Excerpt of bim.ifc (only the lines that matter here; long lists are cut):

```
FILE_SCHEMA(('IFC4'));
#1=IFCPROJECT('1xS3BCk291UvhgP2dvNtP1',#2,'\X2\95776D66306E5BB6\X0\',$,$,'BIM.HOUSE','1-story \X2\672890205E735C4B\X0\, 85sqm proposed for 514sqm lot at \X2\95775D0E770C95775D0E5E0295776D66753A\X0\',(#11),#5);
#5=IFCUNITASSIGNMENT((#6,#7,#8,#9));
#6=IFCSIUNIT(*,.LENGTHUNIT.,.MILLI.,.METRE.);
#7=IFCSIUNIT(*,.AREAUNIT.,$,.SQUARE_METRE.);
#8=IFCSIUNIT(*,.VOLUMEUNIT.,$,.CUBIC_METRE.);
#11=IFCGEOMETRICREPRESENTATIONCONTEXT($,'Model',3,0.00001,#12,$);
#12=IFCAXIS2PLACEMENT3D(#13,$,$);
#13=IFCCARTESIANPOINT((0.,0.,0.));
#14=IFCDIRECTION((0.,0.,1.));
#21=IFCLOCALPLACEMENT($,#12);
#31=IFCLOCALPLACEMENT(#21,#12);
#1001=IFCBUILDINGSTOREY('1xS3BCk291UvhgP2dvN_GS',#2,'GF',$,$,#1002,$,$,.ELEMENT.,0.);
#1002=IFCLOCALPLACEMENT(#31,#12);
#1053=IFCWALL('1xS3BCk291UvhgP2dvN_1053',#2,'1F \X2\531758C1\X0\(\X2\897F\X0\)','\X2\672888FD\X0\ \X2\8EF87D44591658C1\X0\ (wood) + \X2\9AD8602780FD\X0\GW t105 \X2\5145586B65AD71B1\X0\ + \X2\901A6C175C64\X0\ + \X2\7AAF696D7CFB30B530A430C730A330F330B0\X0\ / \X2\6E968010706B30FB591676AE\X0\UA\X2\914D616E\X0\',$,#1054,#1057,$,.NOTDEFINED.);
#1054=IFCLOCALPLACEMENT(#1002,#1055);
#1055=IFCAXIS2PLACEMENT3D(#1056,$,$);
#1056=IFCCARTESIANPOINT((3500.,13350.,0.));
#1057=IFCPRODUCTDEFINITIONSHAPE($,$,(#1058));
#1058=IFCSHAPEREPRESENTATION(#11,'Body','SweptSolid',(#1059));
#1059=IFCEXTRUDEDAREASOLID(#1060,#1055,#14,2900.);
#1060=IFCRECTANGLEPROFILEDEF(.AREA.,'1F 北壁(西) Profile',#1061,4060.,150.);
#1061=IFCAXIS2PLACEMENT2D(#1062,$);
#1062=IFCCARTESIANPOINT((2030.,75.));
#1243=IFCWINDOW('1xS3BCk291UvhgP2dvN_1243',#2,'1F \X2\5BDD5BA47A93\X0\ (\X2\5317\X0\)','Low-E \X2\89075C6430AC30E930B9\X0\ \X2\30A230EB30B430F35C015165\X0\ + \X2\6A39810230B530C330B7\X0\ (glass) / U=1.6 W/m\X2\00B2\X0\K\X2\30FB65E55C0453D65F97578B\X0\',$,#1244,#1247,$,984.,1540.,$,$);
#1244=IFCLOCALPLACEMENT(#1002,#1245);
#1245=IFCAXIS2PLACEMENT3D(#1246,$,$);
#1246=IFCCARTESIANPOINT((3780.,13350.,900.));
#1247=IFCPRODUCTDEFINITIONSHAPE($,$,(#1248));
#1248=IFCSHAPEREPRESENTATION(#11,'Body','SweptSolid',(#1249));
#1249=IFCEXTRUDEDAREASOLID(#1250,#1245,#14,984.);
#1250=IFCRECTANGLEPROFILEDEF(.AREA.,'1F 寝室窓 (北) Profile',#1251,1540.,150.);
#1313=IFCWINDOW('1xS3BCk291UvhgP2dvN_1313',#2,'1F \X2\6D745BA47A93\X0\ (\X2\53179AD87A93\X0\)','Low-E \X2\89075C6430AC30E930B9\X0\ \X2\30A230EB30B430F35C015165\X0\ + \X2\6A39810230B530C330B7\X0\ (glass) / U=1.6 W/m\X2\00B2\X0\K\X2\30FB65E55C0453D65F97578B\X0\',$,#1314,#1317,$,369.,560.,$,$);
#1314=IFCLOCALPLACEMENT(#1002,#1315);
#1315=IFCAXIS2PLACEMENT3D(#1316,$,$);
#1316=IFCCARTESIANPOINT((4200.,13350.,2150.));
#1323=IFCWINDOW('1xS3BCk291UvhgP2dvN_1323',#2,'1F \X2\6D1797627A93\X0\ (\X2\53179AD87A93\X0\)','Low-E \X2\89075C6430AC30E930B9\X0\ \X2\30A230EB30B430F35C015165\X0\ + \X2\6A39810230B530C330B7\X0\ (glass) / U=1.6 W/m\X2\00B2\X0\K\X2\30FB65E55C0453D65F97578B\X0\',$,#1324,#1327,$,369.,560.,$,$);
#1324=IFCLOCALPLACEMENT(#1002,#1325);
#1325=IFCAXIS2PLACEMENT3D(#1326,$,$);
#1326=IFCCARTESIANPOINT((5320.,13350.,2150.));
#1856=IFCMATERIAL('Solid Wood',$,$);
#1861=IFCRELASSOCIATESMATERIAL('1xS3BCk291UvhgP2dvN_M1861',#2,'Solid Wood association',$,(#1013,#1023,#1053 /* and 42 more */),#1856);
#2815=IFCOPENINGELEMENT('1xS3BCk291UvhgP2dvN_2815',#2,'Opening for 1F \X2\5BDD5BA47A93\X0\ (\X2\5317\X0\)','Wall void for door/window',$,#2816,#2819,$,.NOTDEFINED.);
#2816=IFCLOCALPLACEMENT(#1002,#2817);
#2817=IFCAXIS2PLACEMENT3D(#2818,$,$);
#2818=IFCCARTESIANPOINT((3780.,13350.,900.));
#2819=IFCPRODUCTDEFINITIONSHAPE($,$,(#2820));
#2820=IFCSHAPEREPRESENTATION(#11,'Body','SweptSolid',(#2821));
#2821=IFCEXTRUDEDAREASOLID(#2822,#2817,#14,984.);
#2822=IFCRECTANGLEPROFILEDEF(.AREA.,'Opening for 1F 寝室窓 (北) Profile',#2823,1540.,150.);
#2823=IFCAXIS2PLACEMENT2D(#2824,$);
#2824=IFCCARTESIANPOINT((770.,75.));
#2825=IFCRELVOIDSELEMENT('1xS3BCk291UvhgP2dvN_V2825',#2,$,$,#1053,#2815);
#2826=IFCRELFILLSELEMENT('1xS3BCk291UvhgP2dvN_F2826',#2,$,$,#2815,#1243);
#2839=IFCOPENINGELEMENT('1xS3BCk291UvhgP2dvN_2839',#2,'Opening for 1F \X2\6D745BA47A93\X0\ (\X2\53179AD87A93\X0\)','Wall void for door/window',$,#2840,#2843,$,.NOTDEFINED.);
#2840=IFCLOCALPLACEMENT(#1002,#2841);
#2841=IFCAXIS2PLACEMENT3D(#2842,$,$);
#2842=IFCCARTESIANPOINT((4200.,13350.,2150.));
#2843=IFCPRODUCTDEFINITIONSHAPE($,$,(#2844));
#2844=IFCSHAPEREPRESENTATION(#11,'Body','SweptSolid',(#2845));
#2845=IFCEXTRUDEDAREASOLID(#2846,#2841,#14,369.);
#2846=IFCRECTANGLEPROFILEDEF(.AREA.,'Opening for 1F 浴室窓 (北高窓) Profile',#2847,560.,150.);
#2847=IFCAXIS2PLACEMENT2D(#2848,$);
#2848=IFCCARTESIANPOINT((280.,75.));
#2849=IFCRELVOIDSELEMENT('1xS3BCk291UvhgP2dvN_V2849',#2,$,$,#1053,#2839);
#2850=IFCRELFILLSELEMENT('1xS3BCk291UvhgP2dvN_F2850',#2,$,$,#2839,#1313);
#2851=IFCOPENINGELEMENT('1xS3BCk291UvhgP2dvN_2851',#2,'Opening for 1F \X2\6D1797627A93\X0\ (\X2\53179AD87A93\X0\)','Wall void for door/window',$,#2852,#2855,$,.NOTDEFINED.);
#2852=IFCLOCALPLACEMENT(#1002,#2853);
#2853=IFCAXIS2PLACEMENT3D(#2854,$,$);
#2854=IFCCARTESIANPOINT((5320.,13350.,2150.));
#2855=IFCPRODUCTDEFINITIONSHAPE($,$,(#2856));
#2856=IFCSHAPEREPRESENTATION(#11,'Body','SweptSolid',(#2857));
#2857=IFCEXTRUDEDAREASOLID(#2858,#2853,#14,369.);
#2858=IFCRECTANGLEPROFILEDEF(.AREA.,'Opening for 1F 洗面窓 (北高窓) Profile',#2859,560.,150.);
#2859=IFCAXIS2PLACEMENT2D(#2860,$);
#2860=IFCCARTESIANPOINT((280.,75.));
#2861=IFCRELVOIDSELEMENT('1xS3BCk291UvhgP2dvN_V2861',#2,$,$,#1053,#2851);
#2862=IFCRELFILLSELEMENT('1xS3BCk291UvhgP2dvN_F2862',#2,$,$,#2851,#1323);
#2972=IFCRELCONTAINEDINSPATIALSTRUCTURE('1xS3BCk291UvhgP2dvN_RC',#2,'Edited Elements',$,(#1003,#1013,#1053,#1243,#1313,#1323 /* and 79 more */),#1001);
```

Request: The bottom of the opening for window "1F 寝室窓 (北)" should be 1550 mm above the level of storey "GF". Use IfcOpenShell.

```python
import numpy as np
import ifcopenshell
import ifcopenshell.api.geometry
import ifcopenshell.geom
import ifcopenshell.util.element
import ifcopenshell.util.placement
import ifcopenshell.util.shape
import ifcopenshell.util.unit

model = ifcopenshell.open("bim.ifc")
unit_scale = ifcopenshell.util.unit.calculate_unit_scale(model)

window = model.by_guid("1xS3BCk291UvhgP2dvN_1243")
opening = window.FillsVoids[0].RelatingOpeningElement
storey = ifcopenshell.util.element.get_container(window, ifc_class="IfcBuildingStorey")
level = ifcopenshell.util.placement.get_local_placement(storey.ObjectPlacement)[2, 3]

# The opening's origin need not be at the sill, so measure its lowest point.
shape = ifcopenshell.geom.create_shape(ifcopenshell.geom.settings(), opening)
bottom = ifcopenshell.util.shape.get_shape_bottom_elevation(shape, shape.geometry) / unit_scale
dz = level + 1.55 / unit_scale - bottom

shift = np.array([0.0, 0.0, dz])
# The window is not placed relative to its opening, so move both.
for product in (opening, window):
    matrix = ifcopenshell.util.placement.get_local_placement(product.ObjectPlacement)
    matrix[:3, 3] += shift
    ifcopenshell.api.geometry.edit_object_placement(model, product=product, matrix=matrix, is_si=False)

print(f"moved by {dz * unit_scale:+.3f} m")

model.write("bim_updated.ifc")
```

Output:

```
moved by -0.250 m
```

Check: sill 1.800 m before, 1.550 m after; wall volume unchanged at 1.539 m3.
